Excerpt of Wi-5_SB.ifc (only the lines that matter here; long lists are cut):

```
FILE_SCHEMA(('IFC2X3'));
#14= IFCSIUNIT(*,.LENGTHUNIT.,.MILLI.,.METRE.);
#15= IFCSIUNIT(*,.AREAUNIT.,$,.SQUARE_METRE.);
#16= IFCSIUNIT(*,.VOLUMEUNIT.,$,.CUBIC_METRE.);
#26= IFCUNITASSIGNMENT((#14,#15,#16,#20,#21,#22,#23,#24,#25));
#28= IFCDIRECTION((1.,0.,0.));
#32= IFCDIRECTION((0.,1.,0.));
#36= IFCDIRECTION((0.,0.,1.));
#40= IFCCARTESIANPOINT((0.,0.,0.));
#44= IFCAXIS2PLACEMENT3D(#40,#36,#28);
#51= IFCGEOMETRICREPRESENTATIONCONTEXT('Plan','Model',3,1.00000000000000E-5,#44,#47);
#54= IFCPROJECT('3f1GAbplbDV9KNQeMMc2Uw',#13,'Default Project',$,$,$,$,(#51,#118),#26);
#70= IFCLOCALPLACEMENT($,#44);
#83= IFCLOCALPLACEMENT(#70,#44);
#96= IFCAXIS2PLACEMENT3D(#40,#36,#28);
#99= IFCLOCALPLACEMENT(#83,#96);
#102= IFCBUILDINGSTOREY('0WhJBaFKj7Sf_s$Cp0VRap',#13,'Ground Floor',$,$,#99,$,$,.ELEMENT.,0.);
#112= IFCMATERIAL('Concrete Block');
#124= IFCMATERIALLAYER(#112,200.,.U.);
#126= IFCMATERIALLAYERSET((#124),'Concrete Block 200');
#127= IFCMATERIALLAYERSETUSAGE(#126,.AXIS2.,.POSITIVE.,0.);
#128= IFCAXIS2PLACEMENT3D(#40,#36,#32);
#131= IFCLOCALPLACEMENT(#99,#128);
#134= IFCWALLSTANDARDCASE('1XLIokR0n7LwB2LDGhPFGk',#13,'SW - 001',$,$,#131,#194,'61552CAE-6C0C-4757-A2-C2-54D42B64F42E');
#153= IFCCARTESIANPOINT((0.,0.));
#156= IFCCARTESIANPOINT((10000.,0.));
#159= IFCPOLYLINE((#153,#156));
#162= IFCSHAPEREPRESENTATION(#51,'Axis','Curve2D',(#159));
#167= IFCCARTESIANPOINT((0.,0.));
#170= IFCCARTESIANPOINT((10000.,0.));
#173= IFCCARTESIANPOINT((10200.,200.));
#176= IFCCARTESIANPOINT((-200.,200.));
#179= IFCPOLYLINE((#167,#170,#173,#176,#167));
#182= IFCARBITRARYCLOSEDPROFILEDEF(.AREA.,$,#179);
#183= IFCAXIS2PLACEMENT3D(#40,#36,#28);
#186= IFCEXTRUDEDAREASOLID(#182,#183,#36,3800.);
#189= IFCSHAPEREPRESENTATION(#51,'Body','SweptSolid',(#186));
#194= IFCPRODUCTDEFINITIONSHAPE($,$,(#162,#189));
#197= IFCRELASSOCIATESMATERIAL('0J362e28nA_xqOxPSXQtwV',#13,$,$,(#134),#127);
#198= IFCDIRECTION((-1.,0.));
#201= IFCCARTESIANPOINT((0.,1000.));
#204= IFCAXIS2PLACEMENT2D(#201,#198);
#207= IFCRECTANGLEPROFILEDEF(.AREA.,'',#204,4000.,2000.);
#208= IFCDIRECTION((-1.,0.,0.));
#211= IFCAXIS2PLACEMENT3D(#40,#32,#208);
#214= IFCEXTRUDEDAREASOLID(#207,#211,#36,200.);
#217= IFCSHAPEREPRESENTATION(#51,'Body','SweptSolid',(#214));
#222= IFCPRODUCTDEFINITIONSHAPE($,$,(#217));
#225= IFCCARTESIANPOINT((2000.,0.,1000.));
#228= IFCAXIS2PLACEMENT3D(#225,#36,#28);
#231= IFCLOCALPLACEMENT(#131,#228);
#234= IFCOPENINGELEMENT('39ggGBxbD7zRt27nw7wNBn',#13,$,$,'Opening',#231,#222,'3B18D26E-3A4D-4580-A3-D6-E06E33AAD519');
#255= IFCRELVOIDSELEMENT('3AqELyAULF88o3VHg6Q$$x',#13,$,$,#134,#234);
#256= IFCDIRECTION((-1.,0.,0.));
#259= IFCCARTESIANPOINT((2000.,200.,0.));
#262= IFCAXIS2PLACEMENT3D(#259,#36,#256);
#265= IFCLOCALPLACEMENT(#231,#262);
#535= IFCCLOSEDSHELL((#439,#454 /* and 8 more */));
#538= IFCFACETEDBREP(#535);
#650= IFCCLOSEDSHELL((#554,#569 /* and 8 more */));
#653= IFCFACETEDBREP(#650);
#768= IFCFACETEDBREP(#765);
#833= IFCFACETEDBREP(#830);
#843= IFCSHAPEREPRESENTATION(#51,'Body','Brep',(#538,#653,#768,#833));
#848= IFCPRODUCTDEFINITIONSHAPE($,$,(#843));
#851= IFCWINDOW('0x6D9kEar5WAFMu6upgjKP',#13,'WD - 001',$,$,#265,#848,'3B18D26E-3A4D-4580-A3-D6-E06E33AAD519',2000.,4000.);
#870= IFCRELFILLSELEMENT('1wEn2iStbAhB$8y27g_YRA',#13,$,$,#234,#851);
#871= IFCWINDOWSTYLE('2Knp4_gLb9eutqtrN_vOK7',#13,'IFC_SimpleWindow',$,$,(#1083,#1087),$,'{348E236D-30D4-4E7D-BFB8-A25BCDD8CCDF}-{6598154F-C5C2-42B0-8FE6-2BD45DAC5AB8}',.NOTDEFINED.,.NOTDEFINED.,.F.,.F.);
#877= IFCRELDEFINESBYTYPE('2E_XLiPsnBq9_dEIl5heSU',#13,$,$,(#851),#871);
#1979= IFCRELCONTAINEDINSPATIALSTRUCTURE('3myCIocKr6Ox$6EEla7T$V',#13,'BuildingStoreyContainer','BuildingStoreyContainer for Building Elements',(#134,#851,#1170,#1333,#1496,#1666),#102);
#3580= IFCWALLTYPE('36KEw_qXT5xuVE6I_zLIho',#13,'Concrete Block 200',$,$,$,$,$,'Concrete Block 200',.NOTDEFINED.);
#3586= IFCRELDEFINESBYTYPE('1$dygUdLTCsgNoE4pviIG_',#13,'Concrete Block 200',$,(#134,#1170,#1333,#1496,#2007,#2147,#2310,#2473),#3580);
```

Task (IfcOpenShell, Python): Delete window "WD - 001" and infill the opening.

```python
import ifcopenshell
import ifcopenshell.api.feature
import ifcopenshell.api.root
import ifcopenshell.geom
import ifcopenshell.util.shape

model = ifcopenshell.open("Wi-5_SB.ifc")
settings = ifcopenshell.geom.settings()


def volume(element):
    """Net volume in cubic metres, openings subtracted."""
    shape = ifcopenshell.geom.create_shape(settings, element)
    return ifcopenshell.util.shape.get_volume(shape.geometry)


window = model.by_id(851)
opening = window.FillsVoids[0].RelatingOpeningElement
wall = opening.VoidsElements[0].RelatingBuildingElement
before = volume(wall)

ifcopenshell.api.root.remove_product(model, product=window)
ifcopenshell.api.feature.remove_feature(model, feature=opening)

after = volume(wall)

print(f"wall volume {before:.3f} -> {after:.3f} m3")

model.write("Wi-5_SB_edited.ifc")
```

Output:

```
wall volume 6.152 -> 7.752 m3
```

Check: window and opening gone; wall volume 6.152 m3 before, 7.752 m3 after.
